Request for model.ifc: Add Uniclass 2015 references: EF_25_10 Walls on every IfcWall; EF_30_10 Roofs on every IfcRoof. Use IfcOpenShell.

First a look at what the model holds.

```python
import ifcopenshell

model = ifcopenshell.open("model.ifc")
print(model.schema)
print("classifications:", [c.Name for c in model.by_type("IfcClassification")])
for ifc_class in ("IfcDoor", "IfcRoof", "IfcStair", "IfcWall", "IfcWindow"):
    print(ifc_class, len(model.by_type(ifc_class)))
```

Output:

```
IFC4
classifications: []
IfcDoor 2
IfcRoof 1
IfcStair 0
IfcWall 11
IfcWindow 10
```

```python
import ifcopenshell
import ifcopenshell.api.classification

model = ifcopenshell.open("model.ifc")

system = ifcopenshell.api.classification.add_classification(model, classification="Uniclass 2015")

codes = {
    "IfcWall": ("EF_25_10", "Walls"),
    "IfcRoof": ("EF_30_10", "Roofs"),
}
for ifc_class, (code, name) in codes.items():
    products = model.by_type(ifc_class)
    ifcopenshell.api.classification.add_reference(
        model, products=products, classification=system, identification=code, name=name
    )
    print(code, len(products))

model.write("model_v2.ifc")
```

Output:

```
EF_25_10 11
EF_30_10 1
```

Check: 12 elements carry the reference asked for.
